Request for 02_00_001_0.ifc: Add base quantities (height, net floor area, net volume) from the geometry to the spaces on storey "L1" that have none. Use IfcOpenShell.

First a look at what the model holds.

```python
import ifcopenshell
import ifcopenshell.util.element
import ifcopenshell.util.unit

model = ifcopenshell.open("02_00_001_0.ifc")
print(model.schema)
for unit_type in ("LENGTHUNIT", "AREAUNIT", "VOLUMEUNIT"):
    print(unit_type, ifcopenshell.util.unit.calculate_unit_scale(model, unit_type))
storey = next(s for s in model.by_type("IfcBuildingStorey") if s.Name == "L1")
spaces = [e for e in ifcopenshell.util.element.get_decomposition(storey) if e.is_a("IfcSpace")]
for e in sorted(spaces, key=lambda e: e.id()):
    print(e.id(), e.is_a(), e.Name, list(ifcopenshell.util.element.get_psets(e, qtos_only=True)), sep=" | ")
```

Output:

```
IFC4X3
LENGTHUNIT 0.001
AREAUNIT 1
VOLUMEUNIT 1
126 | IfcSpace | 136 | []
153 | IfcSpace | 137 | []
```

```python
import ifcopenshell
import ifcopenshell.api.pset
import ifcopenshell.geom
import ifcopenshell.util.element
import ifcopenshell.util.shape
import ifcopenshell.util.unit

model = ifcopenshell.open("02_00_001_0.ifc")
unit_scale = ifcopenshell.util.unit.calculate_unit_scale(model)
area_scale = ifcopenshell.util.unit.calculate_unit_scale(model, "AREAUNIT")
volume_scale = ifcopenshell.util.unit.calculate_unit_scale(model, "VOLUMEUNIT")
settings = ifcopenshell.geom.settings()

storey = next(s for s in model.by_type("IfcBuildingStorey") if s.Name == "L1")
spaces = [e for e in ifcopenshell.util.element.get_decomposition(storey) if e.is_a("IfcSpace")]

for e in sorted(spaces, key=lambda e: e.id()):
    if ifcopenshell.util.element.get_psets(e, qtos_only=True, should_inherit=False):
        continue
    # Geometry comes back in metres, in the element's own axes.
    shape = ifcopenshell.geom.create_shape(settings, e)
    values = {
        "Height": ifcopenshell.util.shape.get_z(shape.geometry) / unit_scale,
        "NetFloorArea": ifcopenshell.util.shape.get_footprint_area(shape.geometry) / area_scale,
        "NetVolume": ifcopenshell.util.shape.get_volume(shape.geometry) / volume_scale,
    }
    qto = ifcopenshell.api.pset.add_qto(model, product=e, name="Qto_SpaceBaseQuantities")
    ifcopenshell.api.pset.edit_qto(model, qto=qto, properties=values)
    print(e.id(), {k: round(v, 3) for k, v in values.items()})

model.write("02_00_001_0_updated.ifc")
```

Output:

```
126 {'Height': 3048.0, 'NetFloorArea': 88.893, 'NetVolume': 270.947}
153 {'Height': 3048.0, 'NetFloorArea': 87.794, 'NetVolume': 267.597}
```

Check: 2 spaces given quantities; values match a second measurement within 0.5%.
